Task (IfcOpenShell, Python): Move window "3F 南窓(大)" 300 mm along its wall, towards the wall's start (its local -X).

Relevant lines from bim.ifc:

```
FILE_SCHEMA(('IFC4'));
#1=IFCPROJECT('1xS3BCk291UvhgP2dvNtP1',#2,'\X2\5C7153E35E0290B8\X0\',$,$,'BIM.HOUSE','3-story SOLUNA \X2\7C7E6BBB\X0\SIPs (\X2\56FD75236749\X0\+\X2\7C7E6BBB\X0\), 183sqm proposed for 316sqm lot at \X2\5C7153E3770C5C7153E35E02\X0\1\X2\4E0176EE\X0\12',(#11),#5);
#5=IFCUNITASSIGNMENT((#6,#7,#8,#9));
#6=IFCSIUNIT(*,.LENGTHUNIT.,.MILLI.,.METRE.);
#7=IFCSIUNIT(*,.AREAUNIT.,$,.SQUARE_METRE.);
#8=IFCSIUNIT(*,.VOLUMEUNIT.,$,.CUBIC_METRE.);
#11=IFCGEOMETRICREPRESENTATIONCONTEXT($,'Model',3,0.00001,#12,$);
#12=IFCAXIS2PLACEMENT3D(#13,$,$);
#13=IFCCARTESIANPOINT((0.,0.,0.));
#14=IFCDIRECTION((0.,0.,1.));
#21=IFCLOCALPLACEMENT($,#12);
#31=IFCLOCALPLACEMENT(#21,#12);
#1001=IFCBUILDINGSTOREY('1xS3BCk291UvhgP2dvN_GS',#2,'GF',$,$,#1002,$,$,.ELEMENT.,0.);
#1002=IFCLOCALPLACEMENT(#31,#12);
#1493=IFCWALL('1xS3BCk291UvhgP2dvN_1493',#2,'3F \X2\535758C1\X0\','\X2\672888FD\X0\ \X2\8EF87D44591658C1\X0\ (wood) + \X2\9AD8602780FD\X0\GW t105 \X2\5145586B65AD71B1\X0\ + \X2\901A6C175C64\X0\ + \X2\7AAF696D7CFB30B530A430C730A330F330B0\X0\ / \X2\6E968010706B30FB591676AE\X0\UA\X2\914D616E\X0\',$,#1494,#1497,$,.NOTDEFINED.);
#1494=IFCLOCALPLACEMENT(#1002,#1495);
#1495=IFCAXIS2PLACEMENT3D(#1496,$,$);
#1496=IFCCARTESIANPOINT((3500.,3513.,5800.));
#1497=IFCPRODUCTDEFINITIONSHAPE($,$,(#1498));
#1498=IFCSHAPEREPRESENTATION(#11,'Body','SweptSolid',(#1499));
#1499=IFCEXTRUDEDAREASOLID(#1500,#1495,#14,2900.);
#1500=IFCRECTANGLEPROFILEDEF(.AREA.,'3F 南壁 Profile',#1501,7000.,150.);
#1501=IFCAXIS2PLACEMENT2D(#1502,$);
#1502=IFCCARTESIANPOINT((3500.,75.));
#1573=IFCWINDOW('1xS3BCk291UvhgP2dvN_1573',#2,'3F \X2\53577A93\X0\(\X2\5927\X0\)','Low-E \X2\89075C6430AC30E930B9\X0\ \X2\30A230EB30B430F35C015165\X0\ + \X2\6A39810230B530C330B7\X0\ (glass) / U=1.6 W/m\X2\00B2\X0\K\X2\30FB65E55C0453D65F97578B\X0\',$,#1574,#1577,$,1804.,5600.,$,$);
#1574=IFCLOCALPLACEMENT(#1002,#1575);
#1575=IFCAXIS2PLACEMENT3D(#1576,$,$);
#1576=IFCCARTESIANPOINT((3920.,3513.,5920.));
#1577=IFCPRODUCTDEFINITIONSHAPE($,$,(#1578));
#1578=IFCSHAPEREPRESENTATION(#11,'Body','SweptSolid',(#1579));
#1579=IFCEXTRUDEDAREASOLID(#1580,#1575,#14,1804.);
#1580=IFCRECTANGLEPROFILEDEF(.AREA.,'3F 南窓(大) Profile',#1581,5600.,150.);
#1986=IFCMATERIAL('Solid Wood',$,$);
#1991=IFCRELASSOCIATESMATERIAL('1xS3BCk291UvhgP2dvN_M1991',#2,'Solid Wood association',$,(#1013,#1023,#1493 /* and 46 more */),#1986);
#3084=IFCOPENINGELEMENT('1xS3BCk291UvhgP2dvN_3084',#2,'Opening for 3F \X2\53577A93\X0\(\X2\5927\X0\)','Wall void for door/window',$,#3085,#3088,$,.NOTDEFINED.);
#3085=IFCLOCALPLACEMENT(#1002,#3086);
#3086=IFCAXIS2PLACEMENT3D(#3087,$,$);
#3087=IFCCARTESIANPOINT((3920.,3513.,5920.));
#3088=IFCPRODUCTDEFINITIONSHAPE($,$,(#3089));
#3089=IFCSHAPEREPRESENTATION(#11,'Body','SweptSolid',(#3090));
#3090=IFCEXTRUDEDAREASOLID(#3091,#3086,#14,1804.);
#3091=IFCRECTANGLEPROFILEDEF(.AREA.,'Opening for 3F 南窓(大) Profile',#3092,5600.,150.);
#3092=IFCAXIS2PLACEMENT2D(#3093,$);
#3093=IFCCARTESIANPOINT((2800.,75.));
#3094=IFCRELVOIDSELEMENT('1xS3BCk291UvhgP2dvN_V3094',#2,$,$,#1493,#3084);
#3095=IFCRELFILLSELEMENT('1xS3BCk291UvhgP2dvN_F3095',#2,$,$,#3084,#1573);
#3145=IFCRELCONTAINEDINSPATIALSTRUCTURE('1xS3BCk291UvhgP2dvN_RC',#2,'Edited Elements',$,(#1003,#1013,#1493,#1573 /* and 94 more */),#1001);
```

```python
import ifcopenshell
import ifcopenshell.api.geometry
import ifcopenshell.util.placement
import ifcopenshell.util.unit

model = ifcopenshell.open("bim.ifc")
unit_scale = ifcopenshell.util.unit.calculate_unit_scale(model)

window = model.by_guid("1xS3BCk291UvhgP2dvN_1573")
opening = window.FillsVoids[0].RelatingOpeningElement
wall = opening.VoidsElements[0].RelatingBuildingElement

wall_matrix = ifcopenshell.util.placement.get_local_placement(wall.ObjectPlacement)
shift = wall_matrix[:3, 0] * -0.3 / unit_scale
before = ifcopenshell.util.placement.get_local_placement(window.ObjectPlacement)[:3, 3].copy()

# The window is not placed relative to its opening, so move both.
for product in (opening, window):
    matrix = ifcopenshell.util.placement.get_local_placement(product.ObjectPlacement)
    matrix[:3, 3] += shift
    ifcopenshell.api.geometry.edit_object_placement(model, product=product, matrix=matrix, is_si=False)

after = ifcopenshell.util.placement.get_local_placement(window.ObjectPlacement)[:3, 3]
print("window moved by", (after - before).round(3) + 0.0)

model.write("bim_edited.ifc")
```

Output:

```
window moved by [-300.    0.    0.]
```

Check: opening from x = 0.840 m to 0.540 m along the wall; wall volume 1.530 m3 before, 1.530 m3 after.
